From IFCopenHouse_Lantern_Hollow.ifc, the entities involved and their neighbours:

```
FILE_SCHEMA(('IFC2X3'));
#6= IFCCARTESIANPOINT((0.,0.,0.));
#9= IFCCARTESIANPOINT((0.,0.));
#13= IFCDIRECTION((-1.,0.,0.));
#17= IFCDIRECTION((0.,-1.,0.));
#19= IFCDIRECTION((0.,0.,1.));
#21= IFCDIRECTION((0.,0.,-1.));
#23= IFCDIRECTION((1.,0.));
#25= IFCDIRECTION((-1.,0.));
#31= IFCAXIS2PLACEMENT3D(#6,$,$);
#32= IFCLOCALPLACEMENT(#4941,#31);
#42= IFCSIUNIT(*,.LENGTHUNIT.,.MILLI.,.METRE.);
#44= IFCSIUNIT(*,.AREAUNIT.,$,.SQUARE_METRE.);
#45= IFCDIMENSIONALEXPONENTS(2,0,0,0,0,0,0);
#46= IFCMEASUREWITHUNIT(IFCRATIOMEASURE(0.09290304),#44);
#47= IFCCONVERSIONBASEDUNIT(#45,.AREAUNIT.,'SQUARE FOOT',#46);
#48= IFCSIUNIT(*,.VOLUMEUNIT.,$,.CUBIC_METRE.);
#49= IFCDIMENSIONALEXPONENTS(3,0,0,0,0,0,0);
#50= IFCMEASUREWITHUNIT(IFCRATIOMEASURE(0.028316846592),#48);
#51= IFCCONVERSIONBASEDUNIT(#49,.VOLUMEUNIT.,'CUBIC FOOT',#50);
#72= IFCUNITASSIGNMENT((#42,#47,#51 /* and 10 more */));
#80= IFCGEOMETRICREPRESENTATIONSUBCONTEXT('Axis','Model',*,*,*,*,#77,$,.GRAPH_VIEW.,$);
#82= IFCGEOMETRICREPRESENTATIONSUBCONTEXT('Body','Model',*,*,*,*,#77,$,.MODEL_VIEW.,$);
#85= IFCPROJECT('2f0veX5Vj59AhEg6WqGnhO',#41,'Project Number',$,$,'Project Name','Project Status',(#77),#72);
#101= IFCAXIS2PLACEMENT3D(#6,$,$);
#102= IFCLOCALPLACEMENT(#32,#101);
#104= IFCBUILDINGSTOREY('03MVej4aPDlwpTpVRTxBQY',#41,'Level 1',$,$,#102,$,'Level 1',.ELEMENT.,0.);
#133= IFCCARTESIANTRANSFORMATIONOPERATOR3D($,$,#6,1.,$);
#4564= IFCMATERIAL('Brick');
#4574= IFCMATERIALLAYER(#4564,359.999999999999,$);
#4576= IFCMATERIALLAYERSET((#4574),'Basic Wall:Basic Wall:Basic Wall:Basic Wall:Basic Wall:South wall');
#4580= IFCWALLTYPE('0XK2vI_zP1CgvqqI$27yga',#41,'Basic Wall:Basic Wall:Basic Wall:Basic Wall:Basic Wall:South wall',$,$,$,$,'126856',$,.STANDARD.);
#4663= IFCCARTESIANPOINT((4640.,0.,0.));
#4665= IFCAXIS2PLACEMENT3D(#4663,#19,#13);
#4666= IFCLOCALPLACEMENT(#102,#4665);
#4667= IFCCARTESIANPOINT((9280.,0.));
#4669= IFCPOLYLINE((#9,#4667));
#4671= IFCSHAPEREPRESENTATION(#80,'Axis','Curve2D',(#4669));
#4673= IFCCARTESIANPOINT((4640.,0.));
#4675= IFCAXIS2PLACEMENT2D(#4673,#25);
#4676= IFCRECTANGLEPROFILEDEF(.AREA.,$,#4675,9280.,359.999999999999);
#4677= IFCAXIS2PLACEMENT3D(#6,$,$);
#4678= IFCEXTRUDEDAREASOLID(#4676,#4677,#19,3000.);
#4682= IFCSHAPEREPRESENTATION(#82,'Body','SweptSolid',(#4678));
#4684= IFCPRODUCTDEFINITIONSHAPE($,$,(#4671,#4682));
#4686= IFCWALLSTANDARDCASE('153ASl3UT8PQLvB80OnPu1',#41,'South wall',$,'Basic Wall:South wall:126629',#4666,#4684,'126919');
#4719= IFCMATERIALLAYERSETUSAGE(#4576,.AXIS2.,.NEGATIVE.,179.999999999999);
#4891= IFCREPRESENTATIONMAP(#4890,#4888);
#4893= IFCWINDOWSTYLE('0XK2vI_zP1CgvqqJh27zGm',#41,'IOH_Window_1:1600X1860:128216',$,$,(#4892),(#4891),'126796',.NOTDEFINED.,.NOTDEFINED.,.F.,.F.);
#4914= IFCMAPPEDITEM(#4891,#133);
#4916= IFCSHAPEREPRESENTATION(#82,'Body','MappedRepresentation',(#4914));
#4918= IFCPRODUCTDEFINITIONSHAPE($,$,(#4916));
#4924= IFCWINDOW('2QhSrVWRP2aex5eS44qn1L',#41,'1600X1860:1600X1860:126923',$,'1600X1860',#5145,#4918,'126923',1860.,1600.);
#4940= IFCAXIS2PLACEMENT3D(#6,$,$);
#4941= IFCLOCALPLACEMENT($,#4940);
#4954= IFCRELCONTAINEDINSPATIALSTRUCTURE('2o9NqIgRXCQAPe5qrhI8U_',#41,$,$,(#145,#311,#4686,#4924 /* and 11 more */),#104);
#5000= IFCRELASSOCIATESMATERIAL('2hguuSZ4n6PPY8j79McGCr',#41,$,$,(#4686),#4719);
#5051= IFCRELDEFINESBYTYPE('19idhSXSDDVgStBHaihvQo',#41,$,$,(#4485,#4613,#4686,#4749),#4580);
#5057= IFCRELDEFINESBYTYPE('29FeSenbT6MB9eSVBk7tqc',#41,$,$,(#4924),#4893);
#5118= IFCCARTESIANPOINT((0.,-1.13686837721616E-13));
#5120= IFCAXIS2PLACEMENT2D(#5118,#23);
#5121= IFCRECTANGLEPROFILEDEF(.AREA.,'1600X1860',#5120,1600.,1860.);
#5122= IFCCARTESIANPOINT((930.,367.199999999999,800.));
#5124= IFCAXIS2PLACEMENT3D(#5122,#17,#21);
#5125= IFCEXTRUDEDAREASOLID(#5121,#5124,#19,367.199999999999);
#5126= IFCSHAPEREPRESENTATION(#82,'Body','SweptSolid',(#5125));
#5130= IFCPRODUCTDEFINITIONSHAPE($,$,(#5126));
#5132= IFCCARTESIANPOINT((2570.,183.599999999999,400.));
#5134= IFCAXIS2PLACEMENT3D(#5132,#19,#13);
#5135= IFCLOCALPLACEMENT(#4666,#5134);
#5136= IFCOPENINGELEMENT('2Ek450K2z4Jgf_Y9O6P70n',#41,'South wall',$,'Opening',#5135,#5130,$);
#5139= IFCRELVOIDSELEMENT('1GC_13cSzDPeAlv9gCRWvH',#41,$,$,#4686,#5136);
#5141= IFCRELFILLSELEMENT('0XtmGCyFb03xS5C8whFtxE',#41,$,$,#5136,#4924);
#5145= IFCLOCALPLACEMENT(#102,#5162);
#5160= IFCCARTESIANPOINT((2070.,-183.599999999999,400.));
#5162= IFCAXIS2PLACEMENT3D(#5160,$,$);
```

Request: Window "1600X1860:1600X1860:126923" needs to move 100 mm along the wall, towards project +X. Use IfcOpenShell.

```python
import ifcopenshell
import ifcopenshell.api.geometry
import ifcopenshell.util.placement
import ifcopenshell.util.unit

model = ifcopenshell.open("IFCopenHouse_Lantern_Hollow.ifc")
unit_scale = ifcopenshell.util.unit.calculate_unit_scale(model)

window = model.by_guid("2QhSrVWRP2aex5eS44qn1L")
opening = window.FillsVoids[0].RelatingOpeningElement
wall = opening.VoidsElements[0].RelatingBuildingElement

wall_matrix = ifcopenshell.util.placement.get_local_placement(wall.ObjectPlacement)
shift = wall_matrix[:3, 0] * -0.1 / unit_scale
before = ifcopenshell.util.placement.get_local_placement(window.ObjectPlacement)[:3, 3].copy()

# The window is not placed relative to its opening, so move both.
for product in (opening, window):
    matrix = ifcopenshell.util.placement.get_local_placement(product.ObjectPlacement)
    matrix[:3, 3] += shift
    ifcopenshell.api.geometry.edit_object_placement(model, product=product, matrix=matrix, is_si=False)

after = ifcopenshell.util.placement.get_local_placement(window.ObjectPlacement)[:3, 3]
print("window moved by", (after - before).round(3) + 0.0)

model.write("IFCopenHouse_Lantern_Hollow_v2.ifc")
```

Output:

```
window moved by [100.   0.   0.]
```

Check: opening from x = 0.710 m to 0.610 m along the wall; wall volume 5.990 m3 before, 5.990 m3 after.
